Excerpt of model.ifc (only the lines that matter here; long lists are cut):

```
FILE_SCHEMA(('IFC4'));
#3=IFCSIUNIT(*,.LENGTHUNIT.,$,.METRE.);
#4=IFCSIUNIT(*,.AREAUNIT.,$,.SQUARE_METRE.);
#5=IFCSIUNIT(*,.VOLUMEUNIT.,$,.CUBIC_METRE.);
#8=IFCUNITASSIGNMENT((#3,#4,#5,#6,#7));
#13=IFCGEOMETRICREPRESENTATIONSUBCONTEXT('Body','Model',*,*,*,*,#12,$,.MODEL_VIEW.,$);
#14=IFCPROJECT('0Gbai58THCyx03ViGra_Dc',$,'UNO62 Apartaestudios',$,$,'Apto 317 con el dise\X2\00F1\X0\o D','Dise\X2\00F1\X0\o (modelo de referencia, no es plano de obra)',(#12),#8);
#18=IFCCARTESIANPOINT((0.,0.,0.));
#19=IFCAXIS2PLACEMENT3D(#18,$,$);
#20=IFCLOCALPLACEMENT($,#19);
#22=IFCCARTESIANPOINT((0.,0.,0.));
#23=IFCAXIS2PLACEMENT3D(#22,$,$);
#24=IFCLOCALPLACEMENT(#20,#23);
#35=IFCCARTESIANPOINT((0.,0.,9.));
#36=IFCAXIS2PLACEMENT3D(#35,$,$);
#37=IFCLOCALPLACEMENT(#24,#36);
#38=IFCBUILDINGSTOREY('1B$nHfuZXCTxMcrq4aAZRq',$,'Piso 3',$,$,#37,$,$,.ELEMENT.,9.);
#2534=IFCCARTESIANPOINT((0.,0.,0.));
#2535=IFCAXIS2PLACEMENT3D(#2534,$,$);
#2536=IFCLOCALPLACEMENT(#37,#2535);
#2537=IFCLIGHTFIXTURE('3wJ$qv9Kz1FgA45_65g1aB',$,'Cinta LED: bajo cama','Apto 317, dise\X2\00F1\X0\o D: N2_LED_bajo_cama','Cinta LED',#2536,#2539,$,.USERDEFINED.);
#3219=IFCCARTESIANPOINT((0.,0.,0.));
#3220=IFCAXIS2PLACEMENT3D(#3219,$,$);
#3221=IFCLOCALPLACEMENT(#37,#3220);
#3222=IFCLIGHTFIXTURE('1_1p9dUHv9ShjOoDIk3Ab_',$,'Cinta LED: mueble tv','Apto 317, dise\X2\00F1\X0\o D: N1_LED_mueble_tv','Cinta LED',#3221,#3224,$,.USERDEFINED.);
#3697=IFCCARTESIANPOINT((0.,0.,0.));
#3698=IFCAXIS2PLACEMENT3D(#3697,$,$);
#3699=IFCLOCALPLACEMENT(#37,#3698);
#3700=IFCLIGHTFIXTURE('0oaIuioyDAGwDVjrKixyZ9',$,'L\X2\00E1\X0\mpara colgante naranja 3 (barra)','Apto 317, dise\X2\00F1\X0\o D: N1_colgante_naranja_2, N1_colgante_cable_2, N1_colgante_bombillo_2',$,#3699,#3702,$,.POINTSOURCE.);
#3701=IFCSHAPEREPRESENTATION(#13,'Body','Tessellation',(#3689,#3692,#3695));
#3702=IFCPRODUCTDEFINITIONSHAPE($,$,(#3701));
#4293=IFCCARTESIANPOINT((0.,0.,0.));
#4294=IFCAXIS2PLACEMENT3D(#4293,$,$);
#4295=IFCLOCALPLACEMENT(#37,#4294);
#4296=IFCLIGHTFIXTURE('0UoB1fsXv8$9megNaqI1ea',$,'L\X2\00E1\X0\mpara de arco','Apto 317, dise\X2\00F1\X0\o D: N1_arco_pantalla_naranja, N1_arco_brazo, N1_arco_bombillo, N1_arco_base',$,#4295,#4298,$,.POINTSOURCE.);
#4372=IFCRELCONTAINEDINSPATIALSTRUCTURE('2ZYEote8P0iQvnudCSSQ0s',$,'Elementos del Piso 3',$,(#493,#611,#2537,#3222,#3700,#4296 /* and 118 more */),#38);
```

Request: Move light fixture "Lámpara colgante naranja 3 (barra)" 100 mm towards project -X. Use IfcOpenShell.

```python
import ifcopenshell
import ifcopenshell.api.geometry
import ifcopenshell.util.placement

model = ifcopenshell.open("model.ifc")

item = model.by_guid("0oaIuioyDAGwDVjrKixyZ9")
matrix = ifcopenshell.util.placement.get_local_placement(item.ObjectPlacement)
matrix[0, 3] -= 0.1
ifcopenshell.api.geometry.edit_object_placement(model, product=item, matrix=matrix, is_si=False)

print(ifcopenshell.util.placement.get_local_placement(item.ObjectPlacement).round(3) + 0.0)

model.write("model_edited.ifc")
```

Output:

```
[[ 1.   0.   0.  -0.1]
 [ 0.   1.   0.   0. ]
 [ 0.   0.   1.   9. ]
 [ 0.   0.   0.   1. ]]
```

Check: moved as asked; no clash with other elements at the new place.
